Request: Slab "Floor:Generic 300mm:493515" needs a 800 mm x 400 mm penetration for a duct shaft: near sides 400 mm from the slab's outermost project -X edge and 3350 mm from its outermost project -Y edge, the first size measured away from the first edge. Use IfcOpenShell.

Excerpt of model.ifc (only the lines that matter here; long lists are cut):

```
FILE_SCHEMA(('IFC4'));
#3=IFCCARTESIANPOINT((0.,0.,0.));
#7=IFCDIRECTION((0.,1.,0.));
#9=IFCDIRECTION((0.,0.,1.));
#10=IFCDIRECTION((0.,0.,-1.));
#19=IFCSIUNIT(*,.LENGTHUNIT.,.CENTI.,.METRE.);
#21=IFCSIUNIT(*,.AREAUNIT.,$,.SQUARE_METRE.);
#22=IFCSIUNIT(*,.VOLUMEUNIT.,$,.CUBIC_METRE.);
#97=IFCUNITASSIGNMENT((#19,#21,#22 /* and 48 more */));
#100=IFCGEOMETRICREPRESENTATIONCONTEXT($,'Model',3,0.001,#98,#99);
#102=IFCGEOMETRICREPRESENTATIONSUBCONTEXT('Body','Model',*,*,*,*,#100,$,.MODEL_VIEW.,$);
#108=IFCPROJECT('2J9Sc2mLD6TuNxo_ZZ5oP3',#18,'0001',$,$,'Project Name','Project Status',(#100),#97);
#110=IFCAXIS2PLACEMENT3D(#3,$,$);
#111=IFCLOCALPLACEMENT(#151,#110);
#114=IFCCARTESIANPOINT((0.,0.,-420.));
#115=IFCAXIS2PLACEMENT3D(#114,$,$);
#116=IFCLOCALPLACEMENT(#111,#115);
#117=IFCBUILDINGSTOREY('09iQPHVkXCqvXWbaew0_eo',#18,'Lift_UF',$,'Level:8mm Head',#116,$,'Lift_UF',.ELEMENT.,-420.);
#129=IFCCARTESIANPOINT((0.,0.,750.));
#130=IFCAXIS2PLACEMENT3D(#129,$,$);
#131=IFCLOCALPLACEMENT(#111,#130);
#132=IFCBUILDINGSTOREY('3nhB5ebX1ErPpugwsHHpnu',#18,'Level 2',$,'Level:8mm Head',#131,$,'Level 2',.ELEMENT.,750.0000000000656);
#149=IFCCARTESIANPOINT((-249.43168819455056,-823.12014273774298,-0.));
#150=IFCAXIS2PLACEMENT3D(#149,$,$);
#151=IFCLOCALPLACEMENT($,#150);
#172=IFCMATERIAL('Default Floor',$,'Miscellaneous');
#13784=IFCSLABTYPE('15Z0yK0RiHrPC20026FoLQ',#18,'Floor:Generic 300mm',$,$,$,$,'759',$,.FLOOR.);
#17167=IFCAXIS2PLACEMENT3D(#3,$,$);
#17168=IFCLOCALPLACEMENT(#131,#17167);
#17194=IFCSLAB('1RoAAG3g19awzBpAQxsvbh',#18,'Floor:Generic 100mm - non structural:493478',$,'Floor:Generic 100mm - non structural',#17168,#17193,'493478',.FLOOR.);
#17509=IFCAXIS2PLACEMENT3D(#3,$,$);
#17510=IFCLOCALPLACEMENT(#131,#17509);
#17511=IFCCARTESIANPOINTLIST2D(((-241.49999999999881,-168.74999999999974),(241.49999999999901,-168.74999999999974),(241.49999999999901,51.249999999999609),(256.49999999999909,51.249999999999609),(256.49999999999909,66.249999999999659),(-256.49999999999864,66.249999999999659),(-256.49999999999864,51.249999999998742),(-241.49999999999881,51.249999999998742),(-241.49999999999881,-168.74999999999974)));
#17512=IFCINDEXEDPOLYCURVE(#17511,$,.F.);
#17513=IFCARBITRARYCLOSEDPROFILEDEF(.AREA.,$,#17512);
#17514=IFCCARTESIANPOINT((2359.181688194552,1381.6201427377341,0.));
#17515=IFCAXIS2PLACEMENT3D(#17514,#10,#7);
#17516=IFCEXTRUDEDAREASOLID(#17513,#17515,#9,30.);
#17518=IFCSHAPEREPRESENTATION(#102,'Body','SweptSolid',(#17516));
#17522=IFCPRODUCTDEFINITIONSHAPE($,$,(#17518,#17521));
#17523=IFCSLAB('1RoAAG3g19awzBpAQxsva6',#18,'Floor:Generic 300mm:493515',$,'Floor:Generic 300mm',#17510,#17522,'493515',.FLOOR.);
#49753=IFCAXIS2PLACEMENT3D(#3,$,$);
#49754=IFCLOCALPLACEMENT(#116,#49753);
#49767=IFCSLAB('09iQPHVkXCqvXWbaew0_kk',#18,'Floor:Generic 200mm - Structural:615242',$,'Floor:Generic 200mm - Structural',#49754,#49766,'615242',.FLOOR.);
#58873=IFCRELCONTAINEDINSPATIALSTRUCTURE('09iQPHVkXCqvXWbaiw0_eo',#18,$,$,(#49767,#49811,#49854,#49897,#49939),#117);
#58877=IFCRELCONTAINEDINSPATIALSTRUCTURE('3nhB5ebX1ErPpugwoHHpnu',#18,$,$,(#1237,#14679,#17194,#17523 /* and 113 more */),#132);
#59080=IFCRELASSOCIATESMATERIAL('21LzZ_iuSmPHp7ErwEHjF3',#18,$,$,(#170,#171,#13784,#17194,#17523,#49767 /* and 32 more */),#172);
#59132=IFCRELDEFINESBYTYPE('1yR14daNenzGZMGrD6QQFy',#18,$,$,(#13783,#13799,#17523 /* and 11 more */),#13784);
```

```python
import numpy as np
import ifcopenshell
import ifcopenshell.api.feature
import ifcopenshell.api.geometry
import ifcopenshell.api.root
import ifcopenshell.geom
import ifcopenshell.util.placement
import ifcopenshell.util.representation
import ifcopenshell.util.shape
import ifcopenshell.util.unit

model = ifcopenshell.open("model.ifc")
unit_scale = ifcopenshell.util.unit.calculate_unit_scale(model)
settings = ifcopenshell.geom.settings()


def volume(element):
    """Net volume in cubic metres, openings subtracted."""
    shape = ifcopenshell.geom.create_shape(settings, element)
    return ifcopenshell.util.shape.get_volume(shape.geometry)


slab = model.by_guid("1RoAAG3g19awzBpAQxsva6")
before = volume(slab)

# Extent in the slab's own axes, in metres. The edges named are its -X and -Y sides.
slab_shape = ifcopenshell.geom.create_shape(settings, slab)
vertices = ifcopenshell.util.shape.get_vertices(slab_shape.geometry)
x_min, y_min, bottom = vertices.min(axis=0)
top = vertices[:, 2].max()

opening = ifcopenshell.api.root.create_entity(model, ifc_class="IfcOpeningElement", name="Duct shaft opening", predefined_type="OPENING")
context = ifcopenshell.util.representation.get_context(model, "Model", "Body", "MODEL_VIEW")
width, depth = 0.8, 0.4
outline = [(0.0, 0.0), (width, 0.0), (width, depth), (0.0, depth), (0.0, 0.0)]
# Overshoot both faces by 50 mm so the cut is clean.
shape = ifcopenshell.api.geometry.add_slab_representation(
    model, context=context, depth=top - bottom + 0.1, polyline=outline
)
ifcopenshell.api.geometry.assign_representation(model, product=opening, representation=shape)

matrix = ifcopenshell.util.placement.get_local_placement(slab.ObjectPlacement)
matrix[:, 3] = matrix @ np.append(np.array([x_min + 0.4, y_min + 3.35, bottom - 0.05]) / unit_scale, 1.0)
ifcopenshell.api.geometry.edit_object_placement(model, product=opening, matrix=matrix, is_si=False)
ifcopenshell.api.feature.add_feature(model, feature=opening, element=slab)

after = volume(slab)

print(f"slab volume {before:.3f} -> {after:.3f} m3")

model.write("model-out.ifc")
```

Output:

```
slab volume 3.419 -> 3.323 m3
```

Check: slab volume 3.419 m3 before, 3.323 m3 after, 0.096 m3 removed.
